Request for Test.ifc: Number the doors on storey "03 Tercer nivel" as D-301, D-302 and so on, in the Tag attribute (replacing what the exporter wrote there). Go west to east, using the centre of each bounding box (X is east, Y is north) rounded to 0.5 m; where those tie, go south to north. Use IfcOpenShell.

First a look at what the model holds.

```python
import ifcopenshell
import ifcopenshell.util.element
import ifcopenshell.util.placement

model = ifcopenshell.open("Test.ifc")
print(model.schema)
storey = next(s for s in model.by_type("IfcBuildingStorey") if s.Name == "03 Tercer nivel")
doors = [e for e in ifcopenshell.util.element.get_decomposition(storey) if e.is_a("IfcDoor")]
for e in sorted(doors, key=lambda e: e.id()):
    origin = ifcopenshell.util.placement.get_local_placement(e.ObjectPlacement)[:3, 3]
    print(e.id(), e.Tag, e.Name, origin.round(2) + 0.0, sep=" | ")
```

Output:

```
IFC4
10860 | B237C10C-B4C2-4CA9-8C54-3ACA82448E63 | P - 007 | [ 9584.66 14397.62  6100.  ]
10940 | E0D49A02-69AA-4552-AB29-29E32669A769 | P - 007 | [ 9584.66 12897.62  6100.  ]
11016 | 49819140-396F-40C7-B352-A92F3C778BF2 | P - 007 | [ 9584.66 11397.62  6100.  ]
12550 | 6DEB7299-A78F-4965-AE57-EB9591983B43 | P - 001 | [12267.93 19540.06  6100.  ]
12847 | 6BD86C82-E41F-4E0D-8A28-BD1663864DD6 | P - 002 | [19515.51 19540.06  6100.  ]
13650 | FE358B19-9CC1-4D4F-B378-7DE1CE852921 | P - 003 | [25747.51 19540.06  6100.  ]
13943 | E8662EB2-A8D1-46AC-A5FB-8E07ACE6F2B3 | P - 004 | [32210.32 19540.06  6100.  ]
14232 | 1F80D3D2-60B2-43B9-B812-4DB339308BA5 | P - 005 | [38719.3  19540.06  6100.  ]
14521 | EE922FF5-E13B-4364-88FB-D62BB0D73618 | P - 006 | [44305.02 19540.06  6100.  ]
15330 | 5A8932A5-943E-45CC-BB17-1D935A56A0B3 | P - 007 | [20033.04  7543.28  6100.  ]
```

```python
import ifcopenshell
import ifcopenshell.geom
import ifcopenshell.util.element
import ifcopenshell.util.shape

model = ifcopenshell.open("Test.ifc")
settings = ifcopenshell.geom.settings()
settings.set("use-world-coords", True)


def centre(element):
    shape = ifcopenshell.geom.create_shape(settings, element)
    return ifcopenshell.util.shape.get_bbox_centroid(shape.geometry)


storey = next(s for s in model.by_type("IfcBuildingStorey") if s.Name == "03 Tercer nivel")
doors = [e for e in ifcopenshell.util.element.get_decomposition(storey) if e.is_a("IfcDoor")]

# Insertion points can sit at a corner or the storey origin, so sort by the geometry (in metres).
centres = {e: centre(e) for e in doors}
doors.sort(key=lambda e: (round(centres[e][0] / 0.5), centres[e][1]))

for i, e in enumerate(doors, start=1):
    number = f"D-3{i:02d}"
    e.Tag = number
    print(e.id(), number)

model.write("Test-out.ifc")
```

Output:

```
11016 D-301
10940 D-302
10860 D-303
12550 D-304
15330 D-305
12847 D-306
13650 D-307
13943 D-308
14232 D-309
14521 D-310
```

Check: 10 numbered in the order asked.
